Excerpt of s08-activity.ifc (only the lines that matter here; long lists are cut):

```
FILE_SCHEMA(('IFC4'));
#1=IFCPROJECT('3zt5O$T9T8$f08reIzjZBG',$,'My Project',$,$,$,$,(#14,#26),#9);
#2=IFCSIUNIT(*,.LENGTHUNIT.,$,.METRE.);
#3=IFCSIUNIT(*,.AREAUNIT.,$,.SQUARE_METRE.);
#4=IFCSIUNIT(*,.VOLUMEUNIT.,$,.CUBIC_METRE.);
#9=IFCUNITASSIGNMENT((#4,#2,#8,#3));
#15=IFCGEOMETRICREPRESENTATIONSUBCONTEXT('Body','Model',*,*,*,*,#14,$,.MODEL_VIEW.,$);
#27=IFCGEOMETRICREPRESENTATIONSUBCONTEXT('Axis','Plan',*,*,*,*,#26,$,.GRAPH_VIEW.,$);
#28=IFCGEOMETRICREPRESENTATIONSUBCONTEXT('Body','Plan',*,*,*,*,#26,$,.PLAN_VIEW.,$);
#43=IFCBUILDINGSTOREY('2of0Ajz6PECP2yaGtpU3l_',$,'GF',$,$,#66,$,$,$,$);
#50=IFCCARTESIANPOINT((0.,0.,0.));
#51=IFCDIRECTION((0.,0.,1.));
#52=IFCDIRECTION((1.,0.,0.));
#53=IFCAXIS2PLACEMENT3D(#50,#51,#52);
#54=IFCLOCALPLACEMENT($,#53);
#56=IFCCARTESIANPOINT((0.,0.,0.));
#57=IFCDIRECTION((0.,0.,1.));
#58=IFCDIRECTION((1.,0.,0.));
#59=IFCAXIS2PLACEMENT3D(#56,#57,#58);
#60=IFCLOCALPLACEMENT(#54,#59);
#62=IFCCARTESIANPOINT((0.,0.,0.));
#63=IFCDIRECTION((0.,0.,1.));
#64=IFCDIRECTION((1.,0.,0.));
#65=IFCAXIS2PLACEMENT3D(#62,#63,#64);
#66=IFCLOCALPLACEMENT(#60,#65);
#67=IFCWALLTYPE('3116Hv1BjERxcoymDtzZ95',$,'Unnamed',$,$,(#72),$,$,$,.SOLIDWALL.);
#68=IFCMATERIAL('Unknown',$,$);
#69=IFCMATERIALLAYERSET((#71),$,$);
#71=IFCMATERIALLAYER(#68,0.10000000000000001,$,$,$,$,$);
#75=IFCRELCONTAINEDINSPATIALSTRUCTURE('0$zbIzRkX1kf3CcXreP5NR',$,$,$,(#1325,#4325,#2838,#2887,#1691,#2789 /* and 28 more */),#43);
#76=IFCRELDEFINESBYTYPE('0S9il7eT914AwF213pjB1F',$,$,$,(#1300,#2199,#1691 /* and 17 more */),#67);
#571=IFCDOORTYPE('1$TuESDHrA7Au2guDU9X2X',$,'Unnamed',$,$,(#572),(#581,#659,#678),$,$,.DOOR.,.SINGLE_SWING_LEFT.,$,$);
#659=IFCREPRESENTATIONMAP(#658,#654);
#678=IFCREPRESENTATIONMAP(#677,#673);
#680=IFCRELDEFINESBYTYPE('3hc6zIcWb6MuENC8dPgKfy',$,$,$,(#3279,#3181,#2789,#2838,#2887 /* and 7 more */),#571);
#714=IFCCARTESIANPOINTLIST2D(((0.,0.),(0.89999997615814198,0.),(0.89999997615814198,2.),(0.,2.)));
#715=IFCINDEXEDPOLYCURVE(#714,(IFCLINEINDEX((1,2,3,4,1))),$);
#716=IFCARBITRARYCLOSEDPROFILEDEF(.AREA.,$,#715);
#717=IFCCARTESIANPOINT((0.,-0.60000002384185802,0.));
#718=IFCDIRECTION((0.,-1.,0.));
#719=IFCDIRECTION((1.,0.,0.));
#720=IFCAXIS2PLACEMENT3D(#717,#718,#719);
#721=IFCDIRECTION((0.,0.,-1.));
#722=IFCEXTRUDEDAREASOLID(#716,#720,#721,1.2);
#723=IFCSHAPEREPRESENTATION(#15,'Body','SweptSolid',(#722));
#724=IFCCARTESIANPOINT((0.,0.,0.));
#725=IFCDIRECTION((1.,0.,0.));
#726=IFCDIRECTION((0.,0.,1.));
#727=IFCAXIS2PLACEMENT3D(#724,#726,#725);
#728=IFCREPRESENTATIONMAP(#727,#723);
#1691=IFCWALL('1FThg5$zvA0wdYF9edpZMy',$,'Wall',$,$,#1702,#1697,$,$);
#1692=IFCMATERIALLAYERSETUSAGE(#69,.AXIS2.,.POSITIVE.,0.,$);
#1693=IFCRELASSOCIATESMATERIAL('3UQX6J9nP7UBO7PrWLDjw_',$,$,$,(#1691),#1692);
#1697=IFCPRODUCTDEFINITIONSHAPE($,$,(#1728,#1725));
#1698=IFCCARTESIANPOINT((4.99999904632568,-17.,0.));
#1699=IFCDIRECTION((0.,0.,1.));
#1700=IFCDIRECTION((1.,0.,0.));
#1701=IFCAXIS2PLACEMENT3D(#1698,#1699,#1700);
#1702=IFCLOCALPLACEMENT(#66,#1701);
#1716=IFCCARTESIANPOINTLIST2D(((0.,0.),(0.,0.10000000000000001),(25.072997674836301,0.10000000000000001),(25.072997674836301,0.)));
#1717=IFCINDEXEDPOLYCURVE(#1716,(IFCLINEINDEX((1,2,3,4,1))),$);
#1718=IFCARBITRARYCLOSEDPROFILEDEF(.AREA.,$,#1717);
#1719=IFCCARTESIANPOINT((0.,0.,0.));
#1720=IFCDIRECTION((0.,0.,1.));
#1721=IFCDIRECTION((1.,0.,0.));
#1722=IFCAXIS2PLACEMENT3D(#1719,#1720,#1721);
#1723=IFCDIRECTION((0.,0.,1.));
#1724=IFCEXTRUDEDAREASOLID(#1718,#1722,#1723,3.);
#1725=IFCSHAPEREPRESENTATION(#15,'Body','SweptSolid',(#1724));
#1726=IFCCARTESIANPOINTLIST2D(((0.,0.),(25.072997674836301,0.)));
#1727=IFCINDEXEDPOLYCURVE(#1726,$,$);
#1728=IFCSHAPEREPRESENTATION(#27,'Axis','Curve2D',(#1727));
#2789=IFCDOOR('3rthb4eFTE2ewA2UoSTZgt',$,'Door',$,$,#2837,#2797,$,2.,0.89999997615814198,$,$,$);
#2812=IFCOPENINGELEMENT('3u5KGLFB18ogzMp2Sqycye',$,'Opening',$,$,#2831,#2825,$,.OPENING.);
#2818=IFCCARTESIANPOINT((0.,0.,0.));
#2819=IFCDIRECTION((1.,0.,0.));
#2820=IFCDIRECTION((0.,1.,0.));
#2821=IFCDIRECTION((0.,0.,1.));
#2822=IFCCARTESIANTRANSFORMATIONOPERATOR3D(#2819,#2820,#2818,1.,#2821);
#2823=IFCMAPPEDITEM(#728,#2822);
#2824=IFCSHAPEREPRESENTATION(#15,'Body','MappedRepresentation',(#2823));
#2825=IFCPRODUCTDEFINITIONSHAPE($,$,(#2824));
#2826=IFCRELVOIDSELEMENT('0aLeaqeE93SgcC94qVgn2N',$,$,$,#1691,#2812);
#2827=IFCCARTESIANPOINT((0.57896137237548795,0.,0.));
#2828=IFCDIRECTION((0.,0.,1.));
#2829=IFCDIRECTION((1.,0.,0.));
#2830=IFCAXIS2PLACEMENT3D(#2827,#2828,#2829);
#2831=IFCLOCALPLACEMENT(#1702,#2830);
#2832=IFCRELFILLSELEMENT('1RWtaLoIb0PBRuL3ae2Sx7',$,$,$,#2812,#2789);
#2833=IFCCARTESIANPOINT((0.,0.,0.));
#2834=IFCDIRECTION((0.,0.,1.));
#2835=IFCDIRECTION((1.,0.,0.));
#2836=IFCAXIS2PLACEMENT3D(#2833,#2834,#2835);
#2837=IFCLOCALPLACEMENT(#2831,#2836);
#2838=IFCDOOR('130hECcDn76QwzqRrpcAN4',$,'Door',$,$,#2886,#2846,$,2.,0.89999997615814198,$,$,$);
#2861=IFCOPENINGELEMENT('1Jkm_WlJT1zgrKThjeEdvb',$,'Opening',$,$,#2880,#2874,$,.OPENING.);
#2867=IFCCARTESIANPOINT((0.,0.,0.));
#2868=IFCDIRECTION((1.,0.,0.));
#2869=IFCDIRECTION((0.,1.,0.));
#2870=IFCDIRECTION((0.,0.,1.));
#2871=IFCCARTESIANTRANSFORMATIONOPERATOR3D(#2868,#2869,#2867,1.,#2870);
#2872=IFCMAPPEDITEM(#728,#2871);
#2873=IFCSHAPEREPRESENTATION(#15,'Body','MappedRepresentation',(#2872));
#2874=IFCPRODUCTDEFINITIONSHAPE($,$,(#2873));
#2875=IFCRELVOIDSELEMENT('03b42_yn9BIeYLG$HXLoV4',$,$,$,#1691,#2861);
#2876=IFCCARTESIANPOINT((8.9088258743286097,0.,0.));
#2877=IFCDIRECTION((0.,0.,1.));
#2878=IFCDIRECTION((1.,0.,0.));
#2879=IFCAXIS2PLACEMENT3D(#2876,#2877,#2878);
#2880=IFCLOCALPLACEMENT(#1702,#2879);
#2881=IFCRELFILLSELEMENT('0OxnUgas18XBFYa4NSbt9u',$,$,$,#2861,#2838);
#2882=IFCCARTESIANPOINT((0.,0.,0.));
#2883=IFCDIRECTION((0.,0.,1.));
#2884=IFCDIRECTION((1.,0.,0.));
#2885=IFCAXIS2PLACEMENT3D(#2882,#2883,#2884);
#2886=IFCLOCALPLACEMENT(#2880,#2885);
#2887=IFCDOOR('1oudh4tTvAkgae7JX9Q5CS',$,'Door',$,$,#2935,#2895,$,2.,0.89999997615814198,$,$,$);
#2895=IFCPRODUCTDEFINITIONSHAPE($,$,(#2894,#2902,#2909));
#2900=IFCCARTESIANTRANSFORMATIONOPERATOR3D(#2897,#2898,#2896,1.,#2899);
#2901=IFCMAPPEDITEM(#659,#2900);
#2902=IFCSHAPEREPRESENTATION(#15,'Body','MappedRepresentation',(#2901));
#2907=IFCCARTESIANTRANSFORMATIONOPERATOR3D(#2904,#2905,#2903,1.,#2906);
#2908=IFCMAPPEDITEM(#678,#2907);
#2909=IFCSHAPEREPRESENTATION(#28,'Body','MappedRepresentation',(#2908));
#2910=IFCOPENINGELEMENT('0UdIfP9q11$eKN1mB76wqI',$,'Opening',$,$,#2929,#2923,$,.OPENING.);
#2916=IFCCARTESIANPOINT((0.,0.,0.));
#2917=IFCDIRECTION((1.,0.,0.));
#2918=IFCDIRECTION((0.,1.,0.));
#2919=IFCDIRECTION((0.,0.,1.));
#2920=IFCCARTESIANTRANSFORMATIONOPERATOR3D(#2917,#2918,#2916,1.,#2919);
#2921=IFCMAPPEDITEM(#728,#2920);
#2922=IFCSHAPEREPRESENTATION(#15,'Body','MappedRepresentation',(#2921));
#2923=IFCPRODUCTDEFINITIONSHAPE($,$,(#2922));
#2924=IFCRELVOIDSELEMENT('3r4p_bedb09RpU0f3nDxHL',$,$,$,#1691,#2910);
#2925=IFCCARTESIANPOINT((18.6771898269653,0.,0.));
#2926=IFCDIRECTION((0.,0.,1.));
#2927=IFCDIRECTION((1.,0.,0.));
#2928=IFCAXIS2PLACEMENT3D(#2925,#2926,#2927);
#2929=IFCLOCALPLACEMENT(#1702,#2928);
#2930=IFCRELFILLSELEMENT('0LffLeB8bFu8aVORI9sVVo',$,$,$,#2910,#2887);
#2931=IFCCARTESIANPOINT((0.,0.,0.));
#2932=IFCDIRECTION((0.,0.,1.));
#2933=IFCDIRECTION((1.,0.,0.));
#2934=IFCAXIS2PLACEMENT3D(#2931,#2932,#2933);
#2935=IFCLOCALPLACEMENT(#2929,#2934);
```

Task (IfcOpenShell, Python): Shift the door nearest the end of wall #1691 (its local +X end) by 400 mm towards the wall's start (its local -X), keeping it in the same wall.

```python
import ifcopenshell
import ifcopenshell.api.geometry
import ifcopenshell.util.placement
import ifcopenshell.util.unit

model = ifcopenshell.open("s08-activity.ifc")
unit_scale = ifcopenshell.util.unit.calculate_unit_scale(model)

door = model.by_guid("1oudh4tTvAkgae7JX9Q5CS")
opening = door.FillsVoids[0].RelatingOpeningElement
wall = opening.VoidsElements[0].RelatingBuildingElement

wall_matrix = ifcopenshell.util.placement.get_local_placement(wall.ObjectPlacement)
shift = wall_matrix[:3, 0] * -0.4 / unit_scale
before = ifcopenshell.util.placement.get_local_placement(door.ObjectPlacement)[:3, 3].copy()

# The door is placed relative to its opening, so it follows when the opening moves.
matrix = ifcopenshell.util.placement.get_local_placement(opening.ObjectPlacement)
matrix[:3, 3] += shift
ifcopenshell.api.geometry.edit_object_placement(
    model, product=opening, matrix=matrix, is_si=False, should_transform_children=True
)

after = ifcopenshell.util.placement.get_local_placement(door.ObjectPlacement)[:3, 3]
print("door moved by", (after - before).round(3) + 0.0)

model.write("s08-activity_edited.ifc")
```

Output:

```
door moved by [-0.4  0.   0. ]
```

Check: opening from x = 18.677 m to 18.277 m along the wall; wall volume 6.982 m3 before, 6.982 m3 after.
